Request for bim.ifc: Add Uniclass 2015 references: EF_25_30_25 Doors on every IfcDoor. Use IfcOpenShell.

First a look at what the model holds.

```python
import ifcopenshell

model = ifcopenshell.open("bim.ifc")
print(model.schema)
print("classifications:", [c.Name for c in model.by_type("IfcClassification")])
for ifc_class in ("IfcDoor", "IfcRoof", "IfcStair", "IfcWall", "IfcWindow"):
    print(ifc_class, len(model.by_type(ifc_class)))
```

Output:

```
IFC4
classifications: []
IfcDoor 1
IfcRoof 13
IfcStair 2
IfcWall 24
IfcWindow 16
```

```python
import ifcopenshell
import ifcopenshell.api.classification

model = ifcopenshell.open("bim.ifc")

system = ifcopenshell.api.classification.add_classification(model, classification="Uniclass 2015")

codes = {
    "IfcDoor": ("EF_25_30_25", "Doors"),
}
for ifc_class, (code, name) in codes.items():
    products = model.by_type(ifc_class)
    ifcopenshell.api.classification.add_reference(
        model, products=products, classification=system, identification=code, name=name
    )
    print(code, len(products))

model.write("bim_rev.ifc")
```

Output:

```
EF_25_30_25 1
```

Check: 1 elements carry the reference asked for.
